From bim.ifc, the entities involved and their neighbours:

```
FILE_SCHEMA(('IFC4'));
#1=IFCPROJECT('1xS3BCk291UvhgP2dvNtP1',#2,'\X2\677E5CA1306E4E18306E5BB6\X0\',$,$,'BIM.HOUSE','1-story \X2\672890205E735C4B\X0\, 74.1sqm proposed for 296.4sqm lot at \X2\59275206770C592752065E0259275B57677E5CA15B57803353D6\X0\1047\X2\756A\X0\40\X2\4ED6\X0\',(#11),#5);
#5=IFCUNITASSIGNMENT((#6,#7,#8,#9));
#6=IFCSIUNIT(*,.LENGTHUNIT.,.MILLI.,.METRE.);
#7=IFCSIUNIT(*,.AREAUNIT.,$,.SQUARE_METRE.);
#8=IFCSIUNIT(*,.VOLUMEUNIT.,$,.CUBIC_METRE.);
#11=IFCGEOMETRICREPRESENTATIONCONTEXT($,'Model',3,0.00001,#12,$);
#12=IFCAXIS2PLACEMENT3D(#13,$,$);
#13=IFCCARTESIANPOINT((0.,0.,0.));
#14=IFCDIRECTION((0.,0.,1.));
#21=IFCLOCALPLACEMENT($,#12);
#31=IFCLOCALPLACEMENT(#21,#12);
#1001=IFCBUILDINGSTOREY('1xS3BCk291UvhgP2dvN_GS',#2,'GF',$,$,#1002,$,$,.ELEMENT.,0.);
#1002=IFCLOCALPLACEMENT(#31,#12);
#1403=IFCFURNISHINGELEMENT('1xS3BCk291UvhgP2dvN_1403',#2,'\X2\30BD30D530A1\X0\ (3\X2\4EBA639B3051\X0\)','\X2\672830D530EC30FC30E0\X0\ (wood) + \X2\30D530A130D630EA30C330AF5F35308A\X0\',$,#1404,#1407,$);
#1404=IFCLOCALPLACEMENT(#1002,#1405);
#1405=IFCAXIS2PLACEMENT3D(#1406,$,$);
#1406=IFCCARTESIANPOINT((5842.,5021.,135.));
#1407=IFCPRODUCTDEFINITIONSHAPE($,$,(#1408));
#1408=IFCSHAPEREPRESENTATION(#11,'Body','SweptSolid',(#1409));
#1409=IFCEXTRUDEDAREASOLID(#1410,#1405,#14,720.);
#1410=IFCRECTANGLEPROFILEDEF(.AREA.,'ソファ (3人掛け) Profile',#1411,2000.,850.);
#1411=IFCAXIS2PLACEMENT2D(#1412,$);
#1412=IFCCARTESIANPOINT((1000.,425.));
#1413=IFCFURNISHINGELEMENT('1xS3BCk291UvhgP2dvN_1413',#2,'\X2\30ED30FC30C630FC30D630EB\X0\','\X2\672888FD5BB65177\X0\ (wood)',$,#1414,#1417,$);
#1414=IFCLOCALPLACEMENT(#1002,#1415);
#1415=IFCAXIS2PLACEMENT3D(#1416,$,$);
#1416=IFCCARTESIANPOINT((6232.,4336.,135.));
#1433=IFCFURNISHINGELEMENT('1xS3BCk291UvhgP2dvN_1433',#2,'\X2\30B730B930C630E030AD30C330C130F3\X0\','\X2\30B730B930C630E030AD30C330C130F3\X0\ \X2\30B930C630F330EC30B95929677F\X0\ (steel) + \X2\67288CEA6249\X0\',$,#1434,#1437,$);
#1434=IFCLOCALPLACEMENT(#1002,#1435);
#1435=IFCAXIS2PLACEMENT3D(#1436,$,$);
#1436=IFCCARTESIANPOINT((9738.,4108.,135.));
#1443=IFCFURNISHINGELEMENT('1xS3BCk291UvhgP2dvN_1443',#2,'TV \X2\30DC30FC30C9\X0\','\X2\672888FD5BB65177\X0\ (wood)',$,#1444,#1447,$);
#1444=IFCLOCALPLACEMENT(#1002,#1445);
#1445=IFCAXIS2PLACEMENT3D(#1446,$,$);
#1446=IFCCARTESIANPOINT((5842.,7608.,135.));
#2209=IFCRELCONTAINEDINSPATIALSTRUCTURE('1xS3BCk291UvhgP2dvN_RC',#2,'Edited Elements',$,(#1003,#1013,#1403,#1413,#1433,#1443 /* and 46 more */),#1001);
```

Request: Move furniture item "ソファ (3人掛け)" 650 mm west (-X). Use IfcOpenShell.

```python
import ifcopenshell
import ifcopenshell.api.geometry
import ifcopenshell.util.placement

model = ifcopenshell.open("bim.ifc")

item = model.by_id(1403)
matrix = ifcopenshell.util.placement.get_local_placement(item.ObjectPlacement)
matrix[0, 3] -= 650.0
ifcopenshell.api.geometry.edit_object_placement(model, product=item, matrix=matrix, is_si=False)

print(ifcopenshell.util.placement.get_local_placement(item.ObjectPlacement).round(3) + 0.0)

model.write("bim_v2.ifc")
```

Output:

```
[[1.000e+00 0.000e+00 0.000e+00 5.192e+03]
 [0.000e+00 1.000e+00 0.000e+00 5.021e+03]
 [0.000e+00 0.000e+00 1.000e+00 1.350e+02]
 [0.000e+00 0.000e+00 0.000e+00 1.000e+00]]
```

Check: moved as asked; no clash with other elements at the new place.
